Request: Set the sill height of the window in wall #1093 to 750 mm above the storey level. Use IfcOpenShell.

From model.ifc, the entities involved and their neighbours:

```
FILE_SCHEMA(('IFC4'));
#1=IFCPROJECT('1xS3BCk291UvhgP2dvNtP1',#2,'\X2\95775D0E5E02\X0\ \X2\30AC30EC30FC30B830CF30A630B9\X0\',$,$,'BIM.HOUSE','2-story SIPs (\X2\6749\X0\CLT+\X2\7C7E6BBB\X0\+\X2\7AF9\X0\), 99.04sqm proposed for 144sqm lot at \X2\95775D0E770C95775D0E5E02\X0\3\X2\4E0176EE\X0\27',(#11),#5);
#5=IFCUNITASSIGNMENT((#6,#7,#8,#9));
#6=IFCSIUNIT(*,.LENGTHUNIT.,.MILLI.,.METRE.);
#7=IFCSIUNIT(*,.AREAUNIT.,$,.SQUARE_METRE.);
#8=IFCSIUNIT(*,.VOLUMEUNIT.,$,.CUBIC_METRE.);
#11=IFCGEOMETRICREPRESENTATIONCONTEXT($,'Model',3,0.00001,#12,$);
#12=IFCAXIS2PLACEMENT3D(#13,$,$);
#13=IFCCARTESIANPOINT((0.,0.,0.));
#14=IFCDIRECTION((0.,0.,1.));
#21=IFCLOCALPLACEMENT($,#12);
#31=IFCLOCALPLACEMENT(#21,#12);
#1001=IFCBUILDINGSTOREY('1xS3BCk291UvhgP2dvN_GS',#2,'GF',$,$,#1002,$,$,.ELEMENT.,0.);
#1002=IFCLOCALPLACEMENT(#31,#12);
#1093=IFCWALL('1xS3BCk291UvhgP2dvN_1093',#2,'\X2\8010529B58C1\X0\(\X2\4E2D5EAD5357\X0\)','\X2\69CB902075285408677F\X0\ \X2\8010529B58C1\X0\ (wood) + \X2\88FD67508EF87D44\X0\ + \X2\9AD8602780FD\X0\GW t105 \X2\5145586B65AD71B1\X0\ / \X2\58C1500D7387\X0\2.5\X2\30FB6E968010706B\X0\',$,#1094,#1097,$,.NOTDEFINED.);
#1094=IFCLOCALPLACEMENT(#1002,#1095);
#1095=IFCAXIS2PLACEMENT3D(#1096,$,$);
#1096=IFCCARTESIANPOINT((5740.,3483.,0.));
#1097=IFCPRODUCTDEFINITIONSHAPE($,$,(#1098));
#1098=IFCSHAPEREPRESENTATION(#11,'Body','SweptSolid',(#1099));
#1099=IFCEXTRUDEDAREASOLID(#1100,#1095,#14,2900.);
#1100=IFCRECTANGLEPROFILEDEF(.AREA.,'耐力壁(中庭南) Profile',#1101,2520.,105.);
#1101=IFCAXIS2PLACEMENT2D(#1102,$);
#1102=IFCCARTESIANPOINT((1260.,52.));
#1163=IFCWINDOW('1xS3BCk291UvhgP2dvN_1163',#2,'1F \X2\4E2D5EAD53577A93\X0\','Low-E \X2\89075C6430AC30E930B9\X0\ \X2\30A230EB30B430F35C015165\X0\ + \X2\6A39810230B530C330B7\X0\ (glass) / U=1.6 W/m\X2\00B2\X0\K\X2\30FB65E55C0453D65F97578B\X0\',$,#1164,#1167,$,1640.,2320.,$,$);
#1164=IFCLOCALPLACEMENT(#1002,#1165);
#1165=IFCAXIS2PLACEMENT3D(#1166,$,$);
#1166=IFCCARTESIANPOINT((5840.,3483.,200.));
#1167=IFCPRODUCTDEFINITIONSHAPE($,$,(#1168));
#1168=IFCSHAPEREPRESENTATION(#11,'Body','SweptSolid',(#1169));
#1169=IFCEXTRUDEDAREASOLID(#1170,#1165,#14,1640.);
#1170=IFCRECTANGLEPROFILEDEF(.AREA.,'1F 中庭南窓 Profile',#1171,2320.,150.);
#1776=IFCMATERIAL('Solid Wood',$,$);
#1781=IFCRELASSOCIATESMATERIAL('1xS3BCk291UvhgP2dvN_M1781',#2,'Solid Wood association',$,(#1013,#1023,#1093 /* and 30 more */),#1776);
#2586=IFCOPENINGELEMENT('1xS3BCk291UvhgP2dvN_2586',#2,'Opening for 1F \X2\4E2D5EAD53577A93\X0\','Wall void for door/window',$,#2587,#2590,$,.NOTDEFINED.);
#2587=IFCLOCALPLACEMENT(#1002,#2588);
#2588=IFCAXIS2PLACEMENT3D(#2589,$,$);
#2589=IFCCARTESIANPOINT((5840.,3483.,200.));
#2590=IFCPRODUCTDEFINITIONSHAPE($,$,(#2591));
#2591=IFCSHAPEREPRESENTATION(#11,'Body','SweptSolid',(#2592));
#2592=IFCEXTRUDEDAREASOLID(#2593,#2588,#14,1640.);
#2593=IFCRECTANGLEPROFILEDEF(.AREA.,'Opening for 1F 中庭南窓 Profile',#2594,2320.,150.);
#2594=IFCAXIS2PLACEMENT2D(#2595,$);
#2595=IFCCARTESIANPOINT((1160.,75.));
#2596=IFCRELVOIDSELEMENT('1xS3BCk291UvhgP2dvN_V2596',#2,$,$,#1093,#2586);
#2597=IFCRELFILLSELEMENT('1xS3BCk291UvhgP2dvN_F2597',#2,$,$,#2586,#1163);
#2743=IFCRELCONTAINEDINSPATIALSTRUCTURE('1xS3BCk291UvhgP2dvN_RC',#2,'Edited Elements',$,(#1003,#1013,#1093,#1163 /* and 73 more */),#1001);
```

```python
import numpy as np
import ifcopenshell
import ifcopenshell.api.geometry
import ifcopenshell.geom
import ifcopenshell.util.element
import ifcopenshell.util.placement
import ifcopenshell.util.shape
import ifcopenshell.util.unit

model = ifcopenshell.open("model.ifc")
unit_scale = ifcopenshell.util.unit.calculate_unit_scale(model)

window = model.by_id(1163)
opening = window.FillsVoids[0].RelatingOpeningElement
storey = ifcopenshell.util.element.get_container(window, ifc_class="IfcBuildingStorey")
level = ifcopenshell.util.placement.get_local_placement(storey.ObjectPlacement)[2, 3]

# The opening's origin need not be at the sill, so measure its lowest point.
shape = ifcopenshell.geom.create_shape(ifcopenshell.geom.settings(), opening)
bottom = ifcopenshell.util.shape.get_shape_bottom_elevation(shape, shape.geometry) / unit_scale
dz = level + 0.75 / unit_scale - bottom

shift = np.array([0.0, 0.0, dz])
# The window is not placed relative to its opening, so move both.
for product in (opening, window):
    matrix = ifcopenshell.util.placement.get_local_placement(product.ObjectPlacement)
    matrix[:3, 3] += shift
    ifcopenshell.api.geometry.edit_object_placement(model, product=product, matrix=matrix, is_si=False)

print(f"moved by {dz * unit_scale:+.3f} m")

model.write("model_v2.ifc")
```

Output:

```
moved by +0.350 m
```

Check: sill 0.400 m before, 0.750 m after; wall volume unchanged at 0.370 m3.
